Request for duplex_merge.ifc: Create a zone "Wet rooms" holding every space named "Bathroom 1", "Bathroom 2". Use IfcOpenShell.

First a look at what the model holds.

```python
import ifcopenshell

model = ifcopenshell.open("duplex_merge.ifc")
print(model.schema)
seen = {}
for space in model.by_type("IfcSpace"):
    seen[space.LongName] = seen.get(space.LongName, 0) + 1
for name, count in sorted(seen.items(), key=str):
    print(count, "x", name)
print("zones:", [z.Name for z in model.by_type("IfcZone")][:20])
```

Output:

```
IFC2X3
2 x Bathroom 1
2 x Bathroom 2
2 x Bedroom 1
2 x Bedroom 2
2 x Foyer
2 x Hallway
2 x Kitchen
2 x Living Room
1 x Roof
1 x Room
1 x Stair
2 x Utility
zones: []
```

```python
import ifcopenshell
import ifcopenshell.api.group
import ifcopenshell.api.root

model = ifcopenshell.open("duplex_merge.ifc")

names = {"Bathroom 1", "Bathroom 2"}
spaces = [s for s in model.by_type("IfcSpace") if s.LongName in names]

zone = ifcopenshell.api.root.create_entity(model, ifc_class="IfcZone", name="Wet rooms")
ifcopenshell.api.group.assign_group(model, products=spaces, group=zone)
print(len(spaces), "spaces in", zone.Name)

model.write("duplex_merge_updated.ifc")
```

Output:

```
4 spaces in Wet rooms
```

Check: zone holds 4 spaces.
